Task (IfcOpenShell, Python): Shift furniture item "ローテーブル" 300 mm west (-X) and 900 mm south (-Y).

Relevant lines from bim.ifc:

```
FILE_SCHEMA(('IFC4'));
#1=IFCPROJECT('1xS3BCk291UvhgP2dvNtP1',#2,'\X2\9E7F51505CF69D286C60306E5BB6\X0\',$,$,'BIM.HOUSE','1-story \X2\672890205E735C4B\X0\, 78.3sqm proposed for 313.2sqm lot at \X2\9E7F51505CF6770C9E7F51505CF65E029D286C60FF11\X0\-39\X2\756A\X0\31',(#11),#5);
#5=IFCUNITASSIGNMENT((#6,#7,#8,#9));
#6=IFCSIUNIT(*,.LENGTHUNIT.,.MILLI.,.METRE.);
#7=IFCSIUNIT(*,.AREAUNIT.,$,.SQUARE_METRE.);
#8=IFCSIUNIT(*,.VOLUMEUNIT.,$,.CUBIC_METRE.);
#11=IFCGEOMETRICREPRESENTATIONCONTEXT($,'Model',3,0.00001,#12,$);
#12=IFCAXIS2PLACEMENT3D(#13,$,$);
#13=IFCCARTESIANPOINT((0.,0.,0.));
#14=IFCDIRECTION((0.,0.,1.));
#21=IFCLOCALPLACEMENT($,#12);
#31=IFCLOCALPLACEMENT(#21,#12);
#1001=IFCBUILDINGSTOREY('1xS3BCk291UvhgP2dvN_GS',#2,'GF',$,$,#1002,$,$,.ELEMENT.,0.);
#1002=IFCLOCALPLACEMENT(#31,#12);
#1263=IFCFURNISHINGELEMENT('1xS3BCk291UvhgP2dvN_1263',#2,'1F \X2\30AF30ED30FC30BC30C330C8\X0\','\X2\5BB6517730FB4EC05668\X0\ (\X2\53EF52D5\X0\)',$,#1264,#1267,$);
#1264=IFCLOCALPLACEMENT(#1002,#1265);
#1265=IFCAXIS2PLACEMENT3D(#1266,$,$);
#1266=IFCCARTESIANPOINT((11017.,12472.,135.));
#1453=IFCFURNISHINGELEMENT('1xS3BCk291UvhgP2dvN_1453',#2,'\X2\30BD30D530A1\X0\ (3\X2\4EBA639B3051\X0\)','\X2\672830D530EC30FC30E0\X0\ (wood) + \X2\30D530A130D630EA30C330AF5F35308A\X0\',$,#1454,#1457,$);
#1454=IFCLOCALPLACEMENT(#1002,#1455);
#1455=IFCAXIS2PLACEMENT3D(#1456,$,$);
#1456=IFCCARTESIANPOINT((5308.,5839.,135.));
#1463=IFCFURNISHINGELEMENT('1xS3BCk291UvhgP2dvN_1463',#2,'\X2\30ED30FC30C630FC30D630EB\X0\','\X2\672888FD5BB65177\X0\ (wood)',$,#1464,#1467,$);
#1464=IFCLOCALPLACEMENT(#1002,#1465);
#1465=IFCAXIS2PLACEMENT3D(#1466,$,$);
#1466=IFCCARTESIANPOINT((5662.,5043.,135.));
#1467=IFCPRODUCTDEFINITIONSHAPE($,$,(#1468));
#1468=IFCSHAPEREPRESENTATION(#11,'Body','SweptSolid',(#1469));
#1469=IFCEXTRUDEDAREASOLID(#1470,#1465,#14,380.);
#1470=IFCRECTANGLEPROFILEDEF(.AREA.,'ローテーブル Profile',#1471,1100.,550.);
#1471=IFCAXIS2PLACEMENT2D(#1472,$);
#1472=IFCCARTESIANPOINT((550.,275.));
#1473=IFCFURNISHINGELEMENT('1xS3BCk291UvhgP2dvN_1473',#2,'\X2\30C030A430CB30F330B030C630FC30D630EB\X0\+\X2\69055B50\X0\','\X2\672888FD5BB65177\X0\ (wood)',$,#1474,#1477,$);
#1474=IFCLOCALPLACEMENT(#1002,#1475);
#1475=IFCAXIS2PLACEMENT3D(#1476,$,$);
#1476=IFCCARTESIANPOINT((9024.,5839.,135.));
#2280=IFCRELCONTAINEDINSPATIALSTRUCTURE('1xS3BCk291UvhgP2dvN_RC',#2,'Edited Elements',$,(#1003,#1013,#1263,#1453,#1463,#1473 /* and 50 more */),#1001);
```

```python
import ifcopenshell
import ifcopenshell.api.geometry
import ifcopenshell.util.placement
import ifcopenshell.util.unit

model = ifcopenshell.open("bim.ifc")
unit_scale = ifcopenshell.util.unit.calculate_unit_scale(model)

item = model.by_guid("1xS3BCk291UvhgP2dvN_1463")
matrix = ifcopenshell.util.placement.get_local_placement(item.ObjectPlacement)
matrix[0, 3] -= 0.3 / unit_scale
matrix[1, 3] -= 0.9 / unit_scale
ifcopenshell.api.geometry.edit_object_placement(model, product=item, matrix=matrix, is_si=False)

print(ifcopenshell.util.placement.get_local_placement(item.ObjectPlacement).round(3) + 0.0)

model.write("bim_edited.ifc")
```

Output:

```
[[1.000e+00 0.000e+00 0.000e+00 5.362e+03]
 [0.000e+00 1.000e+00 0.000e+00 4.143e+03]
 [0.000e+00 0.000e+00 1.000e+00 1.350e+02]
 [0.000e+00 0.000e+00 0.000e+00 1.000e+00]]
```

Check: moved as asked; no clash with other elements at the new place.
